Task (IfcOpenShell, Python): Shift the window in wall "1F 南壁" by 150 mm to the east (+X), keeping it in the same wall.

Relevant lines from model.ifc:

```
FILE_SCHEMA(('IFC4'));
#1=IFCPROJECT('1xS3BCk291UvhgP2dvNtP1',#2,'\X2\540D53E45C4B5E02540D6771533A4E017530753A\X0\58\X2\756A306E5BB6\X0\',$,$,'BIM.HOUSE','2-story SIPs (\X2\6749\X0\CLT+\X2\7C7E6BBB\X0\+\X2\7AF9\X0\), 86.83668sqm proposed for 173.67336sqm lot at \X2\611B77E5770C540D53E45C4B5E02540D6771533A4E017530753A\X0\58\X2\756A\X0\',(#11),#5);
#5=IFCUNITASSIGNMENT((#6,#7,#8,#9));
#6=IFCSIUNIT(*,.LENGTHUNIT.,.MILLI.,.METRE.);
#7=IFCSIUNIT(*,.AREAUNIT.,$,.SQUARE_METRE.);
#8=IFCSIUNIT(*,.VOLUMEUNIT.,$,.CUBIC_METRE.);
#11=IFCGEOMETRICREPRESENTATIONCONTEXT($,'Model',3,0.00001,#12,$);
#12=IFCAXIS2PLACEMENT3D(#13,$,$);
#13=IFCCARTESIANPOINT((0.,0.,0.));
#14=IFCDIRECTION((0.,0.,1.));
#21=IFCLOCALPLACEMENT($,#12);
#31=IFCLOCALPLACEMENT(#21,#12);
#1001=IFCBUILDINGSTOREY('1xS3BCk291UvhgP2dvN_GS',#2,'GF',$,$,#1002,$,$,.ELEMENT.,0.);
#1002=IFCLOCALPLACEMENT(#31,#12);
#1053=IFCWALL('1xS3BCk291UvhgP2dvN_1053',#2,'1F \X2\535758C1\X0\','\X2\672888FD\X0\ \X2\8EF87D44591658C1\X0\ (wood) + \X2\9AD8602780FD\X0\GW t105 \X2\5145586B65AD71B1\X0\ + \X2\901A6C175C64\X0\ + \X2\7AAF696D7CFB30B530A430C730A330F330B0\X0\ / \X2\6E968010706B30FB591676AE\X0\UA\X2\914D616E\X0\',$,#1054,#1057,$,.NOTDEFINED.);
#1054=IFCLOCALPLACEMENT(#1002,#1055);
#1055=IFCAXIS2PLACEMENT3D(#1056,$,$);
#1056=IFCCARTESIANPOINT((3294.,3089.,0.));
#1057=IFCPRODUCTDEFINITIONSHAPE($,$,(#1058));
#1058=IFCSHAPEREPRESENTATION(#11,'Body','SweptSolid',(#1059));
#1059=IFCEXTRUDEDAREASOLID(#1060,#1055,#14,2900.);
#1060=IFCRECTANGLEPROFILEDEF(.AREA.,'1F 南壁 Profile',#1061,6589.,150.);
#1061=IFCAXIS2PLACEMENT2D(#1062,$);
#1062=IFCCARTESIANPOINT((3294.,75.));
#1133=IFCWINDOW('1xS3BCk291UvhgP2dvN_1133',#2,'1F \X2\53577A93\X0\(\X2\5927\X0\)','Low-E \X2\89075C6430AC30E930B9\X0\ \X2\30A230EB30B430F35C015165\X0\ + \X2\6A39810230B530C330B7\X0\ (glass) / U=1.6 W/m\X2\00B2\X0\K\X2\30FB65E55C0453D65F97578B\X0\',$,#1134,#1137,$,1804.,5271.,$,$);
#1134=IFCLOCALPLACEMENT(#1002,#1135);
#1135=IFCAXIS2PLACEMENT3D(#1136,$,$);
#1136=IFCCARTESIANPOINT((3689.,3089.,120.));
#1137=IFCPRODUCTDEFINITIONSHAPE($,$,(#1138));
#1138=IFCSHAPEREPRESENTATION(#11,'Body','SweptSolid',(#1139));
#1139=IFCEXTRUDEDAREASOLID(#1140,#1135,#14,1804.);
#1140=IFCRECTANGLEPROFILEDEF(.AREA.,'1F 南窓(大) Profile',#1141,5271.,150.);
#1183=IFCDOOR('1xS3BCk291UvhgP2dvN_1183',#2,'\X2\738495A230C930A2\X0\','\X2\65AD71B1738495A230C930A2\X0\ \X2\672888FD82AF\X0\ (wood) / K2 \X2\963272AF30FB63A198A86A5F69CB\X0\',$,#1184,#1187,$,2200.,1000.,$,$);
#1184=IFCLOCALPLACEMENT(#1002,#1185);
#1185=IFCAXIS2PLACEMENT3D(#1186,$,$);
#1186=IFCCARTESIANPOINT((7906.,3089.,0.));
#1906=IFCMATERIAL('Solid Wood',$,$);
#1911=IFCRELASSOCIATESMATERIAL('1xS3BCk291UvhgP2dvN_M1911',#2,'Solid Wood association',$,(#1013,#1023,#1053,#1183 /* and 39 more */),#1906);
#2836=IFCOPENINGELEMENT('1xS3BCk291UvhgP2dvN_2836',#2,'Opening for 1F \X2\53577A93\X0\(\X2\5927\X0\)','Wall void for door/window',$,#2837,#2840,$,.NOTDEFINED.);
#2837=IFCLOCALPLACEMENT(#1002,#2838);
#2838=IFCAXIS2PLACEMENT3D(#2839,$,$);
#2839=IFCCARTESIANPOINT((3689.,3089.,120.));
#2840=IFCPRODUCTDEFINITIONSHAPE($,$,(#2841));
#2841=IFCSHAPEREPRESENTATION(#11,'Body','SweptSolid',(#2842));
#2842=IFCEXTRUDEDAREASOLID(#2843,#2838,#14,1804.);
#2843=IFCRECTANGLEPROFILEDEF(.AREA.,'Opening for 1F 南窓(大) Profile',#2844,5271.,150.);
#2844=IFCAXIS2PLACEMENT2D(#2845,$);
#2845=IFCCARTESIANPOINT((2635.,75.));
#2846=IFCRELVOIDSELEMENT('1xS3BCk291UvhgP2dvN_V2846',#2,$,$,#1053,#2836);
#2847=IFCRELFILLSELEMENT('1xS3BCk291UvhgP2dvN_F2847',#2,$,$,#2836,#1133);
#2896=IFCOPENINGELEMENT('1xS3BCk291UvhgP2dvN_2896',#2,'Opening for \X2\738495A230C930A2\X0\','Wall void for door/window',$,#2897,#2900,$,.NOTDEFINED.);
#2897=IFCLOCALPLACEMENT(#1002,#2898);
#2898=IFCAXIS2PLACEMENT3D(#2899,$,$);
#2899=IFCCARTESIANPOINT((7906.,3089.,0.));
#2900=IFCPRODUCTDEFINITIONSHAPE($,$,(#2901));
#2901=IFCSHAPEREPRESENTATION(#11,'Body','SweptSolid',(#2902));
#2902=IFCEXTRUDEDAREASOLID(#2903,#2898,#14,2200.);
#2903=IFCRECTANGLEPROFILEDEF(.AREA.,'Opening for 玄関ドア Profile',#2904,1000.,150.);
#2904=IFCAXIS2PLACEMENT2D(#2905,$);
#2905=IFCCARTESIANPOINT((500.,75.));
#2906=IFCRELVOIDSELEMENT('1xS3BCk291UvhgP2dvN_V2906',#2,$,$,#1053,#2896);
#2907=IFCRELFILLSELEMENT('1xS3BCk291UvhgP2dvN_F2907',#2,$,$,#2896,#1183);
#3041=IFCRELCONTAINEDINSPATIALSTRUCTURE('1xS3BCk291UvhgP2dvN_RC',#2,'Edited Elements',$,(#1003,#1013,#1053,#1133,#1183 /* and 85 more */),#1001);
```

```python
import ifcopenshell
import ifcopenshell.api.geometry
import ifcopenshell.util.placement

model = ifcopenshell.open("model.ifc")

window = model.by_id(1133)
opening = window.FillsVoids[0].RelatingOpeningElement
wall = opening.VoidsElements[0].RelatingBuildingElement

wall_matrix = ifcopenshell.util.placement.get_local_placement(wall.ObjectPlacement)
shift = wall_matrix[:3, 0] * 150.0
before = ifcopenshell.util.placement.get_local_placement(window.ObjectPlacement)[:3, 3].copy()

# The window is not placed relative to its opening, so move both.
for product in (opening, window):
    matrix = ifcopenshell.util.placement.get_local_placement(product.ObjectPlacement)
    matrix[:3, 3] += shift
    ifcopenshell.api.geometry.edit_object_placement(model, product=product, matrix=matrix, is_si=False)

after = ifcopenshell.util.placement.get_local_placement(window.ObjectPlacement)[:3, 3]
print("window moved by", (after - before).round(3) + 0.0)

model.write("model_rev.ifc")
```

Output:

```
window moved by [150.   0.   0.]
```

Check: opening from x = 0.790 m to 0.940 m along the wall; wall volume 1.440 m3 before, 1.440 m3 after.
